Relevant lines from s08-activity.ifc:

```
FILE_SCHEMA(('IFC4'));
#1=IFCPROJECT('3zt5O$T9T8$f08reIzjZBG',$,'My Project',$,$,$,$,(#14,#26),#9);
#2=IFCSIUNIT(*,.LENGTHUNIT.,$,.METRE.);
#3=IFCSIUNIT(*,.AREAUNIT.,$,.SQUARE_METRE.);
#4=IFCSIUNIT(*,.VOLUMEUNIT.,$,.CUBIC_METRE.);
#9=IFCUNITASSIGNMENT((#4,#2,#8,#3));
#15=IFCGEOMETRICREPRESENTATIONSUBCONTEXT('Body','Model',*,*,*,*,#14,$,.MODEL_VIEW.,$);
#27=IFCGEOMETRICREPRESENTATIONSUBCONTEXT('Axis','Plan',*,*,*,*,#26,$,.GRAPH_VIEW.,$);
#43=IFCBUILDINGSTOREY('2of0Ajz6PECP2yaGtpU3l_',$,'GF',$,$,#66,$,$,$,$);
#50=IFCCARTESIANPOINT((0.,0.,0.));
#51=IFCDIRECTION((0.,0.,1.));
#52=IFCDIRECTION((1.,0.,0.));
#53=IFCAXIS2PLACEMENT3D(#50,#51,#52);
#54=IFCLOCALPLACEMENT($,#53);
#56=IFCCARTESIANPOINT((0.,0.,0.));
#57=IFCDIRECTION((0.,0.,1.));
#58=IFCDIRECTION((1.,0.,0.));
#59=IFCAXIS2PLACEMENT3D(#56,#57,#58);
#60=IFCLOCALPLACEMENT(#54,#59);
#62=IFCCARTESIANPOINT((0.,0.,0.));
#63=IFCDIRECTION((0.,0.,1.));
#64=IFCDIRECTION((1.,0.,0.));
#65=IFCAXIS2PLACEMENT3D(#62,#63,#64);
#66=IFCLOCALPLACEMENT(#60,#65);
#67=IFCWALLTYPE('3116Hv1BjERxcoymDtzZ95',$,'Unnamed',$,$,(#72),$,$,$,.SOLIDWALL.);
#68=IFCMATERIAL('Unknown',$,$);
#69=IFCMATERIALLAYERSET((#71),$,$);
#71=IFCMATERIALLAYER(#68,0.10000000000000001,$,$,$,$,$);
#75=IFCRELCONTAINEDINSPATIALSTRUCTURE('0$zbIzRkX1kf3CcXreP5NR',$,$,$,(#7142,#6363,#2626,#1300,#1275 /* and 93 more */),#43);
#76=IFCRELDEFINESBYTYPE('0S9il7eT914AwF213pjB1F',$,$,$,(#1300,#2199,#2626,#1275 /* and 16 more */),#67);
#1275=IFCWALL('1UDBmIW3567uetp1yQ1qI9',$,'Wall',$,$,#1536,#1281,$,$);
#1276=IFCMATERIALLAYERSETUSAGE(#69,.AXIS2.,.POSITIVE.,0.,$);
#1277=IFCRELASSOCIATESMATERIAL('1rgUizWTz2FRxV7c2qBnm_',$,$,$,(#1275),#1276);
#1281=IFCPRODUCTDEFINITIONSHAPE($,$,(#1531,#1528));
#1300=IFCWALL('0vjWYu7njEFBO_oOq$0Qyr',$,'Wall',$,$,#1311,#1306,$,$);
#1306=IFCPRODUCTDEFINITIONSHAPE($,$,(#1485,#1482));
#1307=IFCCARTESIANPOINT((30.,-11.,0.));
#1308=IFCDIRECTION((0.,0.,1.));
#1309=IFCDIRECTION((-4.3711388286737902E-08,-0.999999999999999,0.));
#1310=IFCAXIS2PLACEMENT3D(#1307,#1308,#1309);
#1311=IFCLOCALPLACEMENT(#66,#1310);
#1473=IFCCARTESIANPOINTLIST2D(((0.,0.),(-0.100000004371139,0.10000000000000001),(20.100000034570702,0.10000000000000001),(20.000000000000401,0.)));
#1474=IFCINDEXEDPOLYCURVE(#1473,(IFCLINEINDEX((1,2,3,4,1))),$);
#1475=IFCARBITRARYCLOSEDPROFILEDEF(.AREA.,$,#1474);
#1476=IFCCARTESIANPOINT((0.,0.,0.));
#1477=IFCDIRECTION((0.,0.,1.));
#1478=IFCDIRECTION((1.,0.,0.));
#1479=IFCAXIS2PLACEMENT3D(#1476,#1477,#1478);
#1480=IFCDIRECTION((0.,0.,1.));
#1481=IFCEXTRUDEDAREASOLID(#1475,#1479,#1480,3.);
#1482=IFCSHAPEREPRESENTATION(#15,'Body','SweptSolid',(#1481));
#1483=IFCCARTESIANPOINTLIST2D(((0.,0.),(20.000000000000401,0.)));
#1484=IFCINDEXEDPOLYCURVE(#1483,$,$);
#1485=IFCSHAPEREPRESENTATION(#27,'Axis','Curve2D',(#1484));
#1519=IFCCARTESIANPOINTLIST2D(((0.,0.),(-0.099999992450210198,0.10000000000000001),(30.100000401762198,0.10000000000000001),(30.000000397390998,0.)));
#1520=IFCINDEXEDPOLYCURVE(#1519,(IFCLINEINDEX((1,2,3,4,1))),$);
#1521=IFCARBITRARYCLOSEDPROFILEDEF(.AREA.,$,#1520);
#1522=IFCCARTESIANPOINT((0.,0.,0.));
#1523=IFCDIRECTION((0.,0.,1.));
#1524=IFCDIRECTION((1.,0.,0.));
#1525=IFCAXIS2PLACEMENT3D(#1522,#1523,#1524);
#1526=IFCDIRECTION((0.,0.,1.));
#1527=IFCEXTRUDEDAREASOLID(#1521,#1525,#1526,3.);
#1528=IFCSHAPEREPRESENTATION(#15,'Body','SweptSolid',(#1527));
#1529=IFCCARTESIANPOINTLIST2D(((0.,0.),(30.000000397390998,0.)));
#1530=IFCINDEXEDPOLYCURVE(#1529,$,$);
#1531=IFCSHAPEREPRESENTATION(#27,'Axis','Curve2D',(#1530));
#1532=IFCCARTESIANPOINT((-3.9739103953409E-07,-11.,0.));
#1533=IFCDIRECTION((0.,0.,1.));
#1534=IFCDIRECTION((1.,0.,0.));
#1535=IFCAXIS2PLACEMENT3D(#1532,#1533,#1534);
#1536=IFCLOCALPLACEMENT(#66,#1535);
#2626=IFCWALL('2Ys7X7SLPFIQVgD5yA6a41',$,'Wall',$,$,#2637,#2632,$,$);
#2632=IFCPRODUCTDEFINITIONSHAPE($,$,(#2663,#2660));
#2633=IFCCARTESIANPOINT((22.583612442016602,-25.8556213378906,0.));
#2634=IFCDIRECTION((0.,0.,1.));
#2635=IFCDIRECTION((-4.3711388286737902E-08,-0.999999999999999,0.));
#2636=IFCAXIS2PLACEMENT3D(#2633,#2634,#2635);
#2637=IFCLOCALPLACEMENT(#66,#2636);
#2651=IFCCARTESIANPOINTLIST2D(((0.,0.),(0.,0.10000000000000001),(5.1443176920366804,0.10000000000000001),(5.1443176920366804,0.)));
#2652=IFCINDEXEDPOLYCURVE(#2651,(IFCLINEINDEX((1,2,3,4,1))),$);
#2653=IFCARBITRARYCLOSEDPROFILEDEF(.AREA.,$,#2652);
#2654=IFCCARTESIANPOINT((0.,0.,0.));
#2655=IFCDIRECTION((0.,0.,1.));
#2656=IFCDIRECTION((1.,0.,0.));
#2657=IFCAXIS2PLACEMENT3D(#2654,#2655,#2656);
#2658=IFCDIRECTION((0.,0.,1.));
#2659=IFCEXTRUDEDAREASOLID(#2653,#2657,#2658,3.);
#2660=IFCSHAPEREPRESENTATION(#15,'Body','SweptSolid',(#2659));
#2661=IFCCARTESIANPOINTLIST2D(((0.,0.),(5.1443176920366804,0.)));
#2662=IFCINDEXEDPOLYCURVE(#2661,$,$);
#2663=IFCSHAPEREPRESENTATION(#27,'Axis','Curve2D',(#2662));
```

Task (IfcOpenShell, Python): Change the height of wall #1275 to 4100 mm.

```python
import ifcopenshell
import ifcopenshell.geom
import ifcopenshell.util.representation
import ifcopenshell.util.shape

model = ifcopenshell.open("s08-activity.ifc")
settings = ifcopenshell.geom.settings()


def volume(element):
    """Net volume in cubic metres, openings subtracted."""
    shape = ifcopenshell.geom.create_shape(settings, element)
    return ifcopenshell.util.shape.get_volume(shape.geometry)


wall = model.by_guid("1UDBmIW3567uetp1yQ1qI9")
before = volume(wall)

body = ifcopenshell.util.representation.get_representation(wall, "Model", "Body")
solid = body.Items[0]
old_height = solid.Depth
solid.Depth = 4.1
after = volume(wall)

print(f"height {old_height:g} -> {solid.Depth:g}, volume {before:.3f} -> {after:.3f} m3")

model.write("s08-activity_updated.ifc")
```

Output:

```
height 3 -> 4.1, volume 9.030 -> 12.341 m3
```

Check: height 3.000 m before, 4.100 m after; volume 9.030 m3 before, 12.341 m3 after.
